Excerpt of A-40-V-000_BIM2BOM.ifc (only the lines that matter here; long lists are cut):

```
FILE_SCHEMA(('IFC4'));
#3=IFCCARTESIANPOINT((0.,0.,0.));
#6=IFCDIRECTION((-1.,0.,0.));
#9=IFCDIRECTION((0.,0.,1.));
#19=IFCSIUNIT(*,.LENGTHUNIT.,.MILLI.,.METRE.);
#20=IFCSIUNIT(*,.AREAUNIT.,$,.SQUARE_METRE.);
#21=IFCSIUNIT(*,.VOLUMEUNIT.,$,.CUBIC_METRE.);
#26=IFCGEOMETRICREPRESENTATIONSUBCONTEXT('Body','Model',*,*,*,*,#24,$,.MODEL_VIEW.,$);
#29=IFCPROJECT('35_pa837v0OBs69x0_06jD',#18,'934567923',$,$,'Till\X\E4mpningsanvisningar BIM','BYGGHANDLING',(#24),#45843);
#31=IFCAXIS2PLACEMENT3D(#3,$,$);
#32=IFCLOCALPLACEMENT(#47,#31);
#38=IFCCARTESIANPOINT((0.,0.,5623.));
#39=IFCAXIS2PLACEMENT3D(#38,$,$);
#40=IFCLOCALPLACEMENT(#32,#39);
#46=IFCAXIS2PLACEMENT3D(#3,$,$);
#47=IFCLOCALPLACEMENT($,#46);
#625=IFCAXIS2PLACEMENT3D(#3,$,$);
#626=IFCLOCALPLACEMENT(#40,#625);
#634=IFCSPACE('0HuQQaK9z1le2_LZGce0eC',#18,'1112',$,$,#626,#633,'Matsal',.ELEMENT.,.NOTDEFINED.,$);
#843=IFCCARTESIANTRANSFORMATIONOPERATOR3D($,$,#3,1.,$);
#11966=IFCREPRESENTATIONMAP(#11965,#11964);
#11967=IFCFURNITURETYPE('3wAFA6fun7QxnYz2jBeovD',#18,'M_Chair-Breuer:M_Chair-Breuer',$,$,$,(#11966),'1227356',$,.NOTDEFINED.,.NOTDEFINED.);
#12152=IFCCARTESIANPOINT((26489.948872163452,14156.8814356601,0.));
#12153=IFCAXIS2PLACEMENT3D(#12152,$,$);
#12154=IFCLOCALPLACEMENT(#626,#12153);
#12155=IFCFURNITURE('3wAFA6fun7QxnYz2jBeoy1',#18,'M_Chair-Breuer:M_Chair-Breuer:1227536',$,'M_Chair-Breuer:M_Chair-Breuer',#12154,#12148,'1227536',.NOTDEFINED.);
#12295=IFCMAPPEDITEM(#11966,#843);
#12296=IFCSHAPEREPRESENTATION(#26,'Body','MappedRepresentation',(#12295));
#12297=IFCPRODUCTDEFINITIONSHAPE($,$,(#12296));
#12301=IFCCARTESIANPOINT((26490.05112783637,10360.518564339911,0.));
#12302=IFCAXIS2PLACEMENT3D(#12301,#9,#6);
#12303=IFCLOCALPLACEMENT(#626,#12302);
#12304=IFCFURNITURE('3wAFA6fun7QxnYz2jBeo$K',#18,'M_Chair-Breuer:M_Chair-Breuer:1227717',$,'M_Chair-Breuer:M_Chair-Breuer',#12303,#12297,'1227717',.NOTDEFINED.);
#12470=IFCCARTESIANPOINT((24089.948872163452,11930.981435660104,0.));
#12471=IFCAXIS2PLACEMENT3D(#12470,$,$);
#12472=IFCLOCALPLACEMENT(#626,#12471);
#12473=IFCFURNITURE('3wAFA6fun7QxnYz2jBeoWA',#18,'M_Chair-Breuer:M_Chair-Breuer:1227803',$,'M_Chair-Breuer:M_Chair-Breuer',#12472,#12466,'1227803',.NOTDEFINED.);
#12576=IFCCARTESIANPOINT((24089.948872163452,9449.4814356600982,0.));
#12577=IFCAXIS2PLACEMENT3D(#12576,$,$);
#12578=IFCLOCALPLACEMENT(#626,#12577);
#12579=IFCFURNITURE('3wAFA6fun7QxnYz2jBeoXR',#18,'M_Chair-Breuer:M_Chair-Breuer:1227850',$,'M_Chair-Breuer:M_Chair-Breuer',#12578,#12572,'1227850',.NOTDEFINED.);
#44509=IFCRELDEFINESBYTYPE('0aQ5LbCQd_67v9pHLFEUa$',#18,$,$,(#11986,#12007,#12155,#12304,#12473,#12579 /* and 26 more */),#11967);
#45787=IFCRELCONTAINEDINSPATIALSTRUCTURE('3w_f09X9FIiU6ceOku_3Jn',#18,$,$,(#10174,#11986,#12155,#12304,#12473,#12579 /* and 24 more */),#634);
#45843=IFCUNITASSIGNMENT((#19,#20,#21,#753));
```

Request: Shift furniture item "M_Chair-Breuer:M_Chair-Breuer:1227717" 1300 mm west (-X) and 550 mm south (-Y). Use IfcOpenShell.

```python
import ifcopenshell
import ifcopenshell.api.geometry
import ifcopenshell.util.placement
import ifcopenshell.util.unit

model = ifcopenshell.open("A-40-V-000_BIM2BOM.ifc")
unit_scale = ifcopenshell.util.unit.calculate_unit_scale(model)

item = model.by_id(12304)
matrix = ifcopenshell.util.placement.get_local_placement(item.ObjectPlacement)
matrix[0, 3] -= 1.3 / unit_scale
matrix[1, 3] -= 0.55 / unit_scale
ifcopenshell.api.geometry.edit_object_placement(model, product=item, matrix=matrix, is_si=False)

print(ifcopenshell.util.placement.get_local_placement(item.ObjectPlacement).round(3) + 0.0)

model.write("A-40-V-000_BIM2BOM-out.ifc")
```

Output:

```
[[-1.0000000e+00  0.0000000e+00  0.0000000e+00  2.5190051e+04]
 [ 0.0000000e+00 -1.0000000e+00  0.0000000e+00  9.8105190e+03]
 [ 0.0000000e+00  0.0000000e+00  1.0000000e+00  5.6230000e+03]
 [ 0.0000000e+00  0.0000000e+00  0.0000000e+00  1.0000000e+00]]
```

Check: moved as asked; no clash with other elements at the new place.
